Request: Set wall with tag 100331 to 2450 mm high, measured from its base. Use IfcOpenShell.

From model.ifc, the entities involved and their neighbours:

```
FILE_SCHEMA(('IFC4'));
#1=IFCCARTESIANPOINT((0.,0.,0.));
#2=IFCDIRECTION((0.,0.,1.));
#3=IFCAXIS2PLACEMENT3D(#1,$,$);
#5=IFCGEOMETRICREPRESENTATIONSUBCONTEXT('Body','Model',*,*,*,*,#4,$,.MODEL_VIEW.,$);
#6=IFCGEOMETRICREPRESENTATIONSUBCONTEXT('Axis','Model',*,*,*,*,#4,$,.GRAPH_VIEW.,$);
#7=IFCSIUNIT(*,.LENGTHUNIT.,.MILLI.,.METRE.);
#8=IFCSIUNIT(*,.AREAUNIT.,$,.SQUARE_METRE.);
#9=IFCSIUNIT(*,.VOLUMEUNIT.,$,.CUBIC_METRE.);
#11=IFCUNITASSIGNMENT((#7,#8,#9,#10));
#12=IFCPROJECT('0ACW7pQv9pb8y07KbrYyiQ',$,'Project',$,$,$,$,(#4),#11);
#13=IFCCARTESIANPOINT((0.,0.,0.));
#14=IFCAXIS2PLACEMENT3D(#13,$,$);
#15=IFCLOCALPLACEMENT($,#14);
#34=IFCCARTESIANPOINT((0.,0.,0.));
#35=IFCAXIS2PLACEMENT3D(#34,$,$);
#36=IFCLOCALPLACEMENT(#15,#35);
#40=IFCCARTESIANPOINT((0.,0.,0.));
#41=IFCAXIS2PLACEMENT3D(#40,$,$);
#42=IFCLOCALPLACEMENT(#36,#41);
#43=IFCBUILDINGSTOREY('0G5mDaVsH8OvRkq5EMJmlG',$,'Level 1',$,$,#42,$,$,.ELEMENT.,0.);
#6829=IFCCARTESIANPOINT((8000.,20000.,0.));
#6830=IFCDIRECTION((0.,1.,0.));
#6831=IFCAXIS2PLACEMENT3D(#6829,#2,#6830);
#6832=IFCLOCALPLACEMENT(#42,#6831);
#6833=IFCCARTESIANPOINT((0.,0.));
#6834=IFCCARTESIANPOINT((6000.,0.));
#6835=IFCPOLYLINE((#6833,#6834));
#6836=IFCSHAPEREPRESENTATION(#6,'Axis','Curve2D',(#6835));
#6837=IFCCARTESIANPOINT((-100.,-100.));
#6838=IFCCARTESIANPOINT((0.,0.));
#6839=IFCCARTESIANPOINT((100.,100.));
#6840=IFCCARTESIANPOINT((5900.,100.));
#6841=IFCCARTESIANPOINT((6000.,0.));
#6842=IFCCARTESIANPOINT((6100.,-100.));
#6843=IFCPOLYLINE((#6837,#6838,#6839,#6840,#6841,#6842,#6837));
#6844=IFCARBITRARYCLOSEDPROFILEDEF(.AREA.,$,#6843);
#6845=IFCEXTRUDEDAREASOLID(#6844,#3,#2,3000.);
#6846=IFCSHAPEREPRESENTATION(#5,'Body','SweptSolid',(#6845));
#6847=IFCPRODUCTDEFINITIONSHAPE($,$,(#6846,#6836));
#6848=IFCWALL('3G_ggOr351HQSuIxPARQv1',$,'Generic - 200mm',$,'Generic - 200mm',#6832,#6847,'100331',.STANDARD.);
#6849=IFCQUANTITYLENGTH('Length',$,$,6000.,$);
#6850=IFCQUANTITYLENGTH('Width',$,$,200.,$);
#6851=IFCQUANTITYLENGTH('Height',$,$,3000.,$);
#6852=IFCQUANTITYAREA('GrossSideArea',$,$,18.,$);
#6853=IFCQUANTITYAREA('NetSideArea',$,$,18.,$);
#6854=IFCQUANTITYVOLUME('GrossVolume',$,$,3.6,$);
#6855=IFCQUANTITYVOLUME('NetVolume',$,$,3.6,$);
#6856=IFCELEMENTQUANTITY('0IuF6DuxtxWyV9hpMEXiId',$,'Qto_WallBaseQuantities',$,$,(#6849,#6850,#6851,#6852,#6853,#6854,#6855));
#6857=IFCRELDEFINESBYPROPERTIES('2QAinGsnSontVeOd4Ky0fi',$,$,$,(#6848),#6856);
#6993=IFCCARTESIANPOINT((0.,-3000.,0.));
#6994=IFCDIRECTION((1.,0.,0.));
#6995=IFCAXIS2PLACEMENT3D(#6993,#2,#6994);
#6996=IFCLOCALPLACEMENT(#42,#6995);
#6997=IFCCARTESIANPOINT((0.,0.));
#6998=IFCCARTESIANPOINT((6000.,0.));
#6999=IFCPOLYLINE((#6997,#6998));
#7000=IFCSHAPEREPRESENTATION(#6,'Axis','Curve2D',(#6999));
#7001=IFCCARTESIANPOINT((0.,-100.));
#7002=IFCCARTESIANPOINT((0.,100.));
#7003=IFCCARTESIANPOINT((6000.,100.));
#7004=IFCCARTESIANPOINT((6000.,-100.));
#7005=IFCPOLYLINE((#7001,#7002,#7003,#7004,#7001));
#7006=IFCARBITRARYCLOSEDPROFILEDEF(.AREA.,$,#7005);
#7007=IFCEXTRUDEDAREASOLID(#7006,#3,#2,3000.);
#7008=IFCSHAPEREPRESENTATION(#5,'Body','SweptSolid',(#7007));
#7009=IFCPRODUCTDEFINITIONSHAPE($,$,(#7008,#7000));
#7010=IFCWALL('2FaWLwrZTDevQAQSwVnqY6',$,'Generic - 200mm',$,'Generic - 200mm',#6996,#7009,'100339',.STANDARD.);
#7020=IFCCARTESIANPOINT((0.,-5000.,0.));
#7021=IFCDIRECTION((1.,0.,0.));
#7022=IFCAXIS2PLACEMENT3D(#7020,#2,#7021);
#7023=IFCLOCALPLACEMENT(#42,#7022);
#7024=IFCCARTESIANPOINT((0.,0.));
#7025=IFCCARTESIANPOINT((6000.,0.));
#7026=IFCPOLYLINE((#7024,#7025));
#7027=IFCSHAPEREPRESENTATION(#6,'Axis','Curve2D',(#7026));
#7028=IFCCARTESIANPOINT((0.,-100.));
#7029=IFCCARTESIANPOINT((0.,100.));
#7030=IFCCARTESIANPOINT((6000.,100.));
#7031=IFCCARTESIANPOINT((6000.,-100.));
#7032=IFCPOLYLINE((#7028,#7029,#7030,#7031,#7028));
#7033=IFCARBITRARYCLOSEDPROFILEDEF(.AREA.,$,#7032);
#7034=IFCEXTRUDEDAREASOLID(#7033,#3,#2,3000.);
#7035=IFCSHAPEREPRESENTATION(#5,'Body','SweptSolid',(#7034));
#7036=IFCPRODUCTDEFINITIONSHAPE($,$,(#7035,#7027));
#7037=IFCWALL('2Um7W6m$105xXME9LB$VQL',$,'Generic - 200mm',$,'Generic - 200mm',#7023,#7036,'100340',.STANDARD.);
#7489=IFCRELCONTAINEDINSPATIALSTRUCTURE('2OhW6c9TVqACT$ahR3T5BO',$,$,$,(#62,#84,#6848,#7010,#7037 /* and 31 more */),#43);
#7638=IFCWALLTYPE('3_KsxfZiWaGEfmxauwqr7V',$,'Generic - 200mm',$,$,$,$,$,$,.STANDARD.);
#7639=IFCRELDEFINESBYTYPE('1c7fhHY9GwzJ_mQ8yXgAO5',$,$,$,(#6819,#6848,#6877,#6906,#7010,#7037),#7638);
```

```python
import ifcopenshell
import ifcopenshell.api.pset
import ifcopenshell.geom
import ifcopenshell.util.element
import ifcopenshell.util.representation
import ifcopenshell.util.shape
import ifcopenshell.util.unit

model = ifcopenshell.open("model.ifc")
unit_scale = ifcopenshell.util.unit.calculate_unit_scale(model)
area_scale = ifcopenshell.util.unit.calculate_unit_scale(model, "AREAUNIT")
volume_scale = ifcopenshell.util.unit.calculate_unit_scale(model, "VOLUMEUNIT")
settings = ifcopenshell.geom.settings()


def volume(element):
    """Net volume in cubic metres, openings subtracted."""
    shape = ifcopenshell.geom.create_shape(settings, element)
    return ifcopenshell.util.shape.get_volume(shape.geometry)


wall = model.by_guid("3G_ggOr351HQSuIxPARQv1")
before = volume(wall)

body = ifcopenshell.util.representation.get_representation(wall, "Model", "Body")
solid = body.Items[0]
old_height = solid.Depth
solid.Depth = 2.45 / unit_scale
after = volume(wall)
thickness = 0.2  # wall thickness in metres

# Update the stored height, areas and volumes.
qto = model.by_id(ifcopenshell.util.element.get_pset(wall, "Qto_WallBaseQuantities", should_inherit=False)["id"])
ifcopenshell.api.pset.edit_qto(model, qto=qto, properties={
    "Height": solid.Depth,
    "GrossSideArea": ifcopenshell.util.element.get_pset(wall, "Qto_WallBaseQuantities", "GrossSideArea") * solid.Depth / old_height,
    "NetSideArea": after / thickness / area_scale,
    "GrossVolume": ifcopenshell.util.element.get_pset(wall, "Qto_WallBaseQuantities", "GrossVolume") * solid.Depth / old_height,
    "NetVolume": after / volume_scale,
})

print(f"height {old_height:g} -> {solid.Depth:g}, volume {before:.3f} -> {after:.3f} m3")

model.write("model_rev.ifc")
```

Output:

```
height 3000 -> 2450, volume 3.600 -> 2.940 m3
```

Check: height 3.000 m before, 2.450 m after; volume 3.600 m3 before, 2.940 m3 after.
